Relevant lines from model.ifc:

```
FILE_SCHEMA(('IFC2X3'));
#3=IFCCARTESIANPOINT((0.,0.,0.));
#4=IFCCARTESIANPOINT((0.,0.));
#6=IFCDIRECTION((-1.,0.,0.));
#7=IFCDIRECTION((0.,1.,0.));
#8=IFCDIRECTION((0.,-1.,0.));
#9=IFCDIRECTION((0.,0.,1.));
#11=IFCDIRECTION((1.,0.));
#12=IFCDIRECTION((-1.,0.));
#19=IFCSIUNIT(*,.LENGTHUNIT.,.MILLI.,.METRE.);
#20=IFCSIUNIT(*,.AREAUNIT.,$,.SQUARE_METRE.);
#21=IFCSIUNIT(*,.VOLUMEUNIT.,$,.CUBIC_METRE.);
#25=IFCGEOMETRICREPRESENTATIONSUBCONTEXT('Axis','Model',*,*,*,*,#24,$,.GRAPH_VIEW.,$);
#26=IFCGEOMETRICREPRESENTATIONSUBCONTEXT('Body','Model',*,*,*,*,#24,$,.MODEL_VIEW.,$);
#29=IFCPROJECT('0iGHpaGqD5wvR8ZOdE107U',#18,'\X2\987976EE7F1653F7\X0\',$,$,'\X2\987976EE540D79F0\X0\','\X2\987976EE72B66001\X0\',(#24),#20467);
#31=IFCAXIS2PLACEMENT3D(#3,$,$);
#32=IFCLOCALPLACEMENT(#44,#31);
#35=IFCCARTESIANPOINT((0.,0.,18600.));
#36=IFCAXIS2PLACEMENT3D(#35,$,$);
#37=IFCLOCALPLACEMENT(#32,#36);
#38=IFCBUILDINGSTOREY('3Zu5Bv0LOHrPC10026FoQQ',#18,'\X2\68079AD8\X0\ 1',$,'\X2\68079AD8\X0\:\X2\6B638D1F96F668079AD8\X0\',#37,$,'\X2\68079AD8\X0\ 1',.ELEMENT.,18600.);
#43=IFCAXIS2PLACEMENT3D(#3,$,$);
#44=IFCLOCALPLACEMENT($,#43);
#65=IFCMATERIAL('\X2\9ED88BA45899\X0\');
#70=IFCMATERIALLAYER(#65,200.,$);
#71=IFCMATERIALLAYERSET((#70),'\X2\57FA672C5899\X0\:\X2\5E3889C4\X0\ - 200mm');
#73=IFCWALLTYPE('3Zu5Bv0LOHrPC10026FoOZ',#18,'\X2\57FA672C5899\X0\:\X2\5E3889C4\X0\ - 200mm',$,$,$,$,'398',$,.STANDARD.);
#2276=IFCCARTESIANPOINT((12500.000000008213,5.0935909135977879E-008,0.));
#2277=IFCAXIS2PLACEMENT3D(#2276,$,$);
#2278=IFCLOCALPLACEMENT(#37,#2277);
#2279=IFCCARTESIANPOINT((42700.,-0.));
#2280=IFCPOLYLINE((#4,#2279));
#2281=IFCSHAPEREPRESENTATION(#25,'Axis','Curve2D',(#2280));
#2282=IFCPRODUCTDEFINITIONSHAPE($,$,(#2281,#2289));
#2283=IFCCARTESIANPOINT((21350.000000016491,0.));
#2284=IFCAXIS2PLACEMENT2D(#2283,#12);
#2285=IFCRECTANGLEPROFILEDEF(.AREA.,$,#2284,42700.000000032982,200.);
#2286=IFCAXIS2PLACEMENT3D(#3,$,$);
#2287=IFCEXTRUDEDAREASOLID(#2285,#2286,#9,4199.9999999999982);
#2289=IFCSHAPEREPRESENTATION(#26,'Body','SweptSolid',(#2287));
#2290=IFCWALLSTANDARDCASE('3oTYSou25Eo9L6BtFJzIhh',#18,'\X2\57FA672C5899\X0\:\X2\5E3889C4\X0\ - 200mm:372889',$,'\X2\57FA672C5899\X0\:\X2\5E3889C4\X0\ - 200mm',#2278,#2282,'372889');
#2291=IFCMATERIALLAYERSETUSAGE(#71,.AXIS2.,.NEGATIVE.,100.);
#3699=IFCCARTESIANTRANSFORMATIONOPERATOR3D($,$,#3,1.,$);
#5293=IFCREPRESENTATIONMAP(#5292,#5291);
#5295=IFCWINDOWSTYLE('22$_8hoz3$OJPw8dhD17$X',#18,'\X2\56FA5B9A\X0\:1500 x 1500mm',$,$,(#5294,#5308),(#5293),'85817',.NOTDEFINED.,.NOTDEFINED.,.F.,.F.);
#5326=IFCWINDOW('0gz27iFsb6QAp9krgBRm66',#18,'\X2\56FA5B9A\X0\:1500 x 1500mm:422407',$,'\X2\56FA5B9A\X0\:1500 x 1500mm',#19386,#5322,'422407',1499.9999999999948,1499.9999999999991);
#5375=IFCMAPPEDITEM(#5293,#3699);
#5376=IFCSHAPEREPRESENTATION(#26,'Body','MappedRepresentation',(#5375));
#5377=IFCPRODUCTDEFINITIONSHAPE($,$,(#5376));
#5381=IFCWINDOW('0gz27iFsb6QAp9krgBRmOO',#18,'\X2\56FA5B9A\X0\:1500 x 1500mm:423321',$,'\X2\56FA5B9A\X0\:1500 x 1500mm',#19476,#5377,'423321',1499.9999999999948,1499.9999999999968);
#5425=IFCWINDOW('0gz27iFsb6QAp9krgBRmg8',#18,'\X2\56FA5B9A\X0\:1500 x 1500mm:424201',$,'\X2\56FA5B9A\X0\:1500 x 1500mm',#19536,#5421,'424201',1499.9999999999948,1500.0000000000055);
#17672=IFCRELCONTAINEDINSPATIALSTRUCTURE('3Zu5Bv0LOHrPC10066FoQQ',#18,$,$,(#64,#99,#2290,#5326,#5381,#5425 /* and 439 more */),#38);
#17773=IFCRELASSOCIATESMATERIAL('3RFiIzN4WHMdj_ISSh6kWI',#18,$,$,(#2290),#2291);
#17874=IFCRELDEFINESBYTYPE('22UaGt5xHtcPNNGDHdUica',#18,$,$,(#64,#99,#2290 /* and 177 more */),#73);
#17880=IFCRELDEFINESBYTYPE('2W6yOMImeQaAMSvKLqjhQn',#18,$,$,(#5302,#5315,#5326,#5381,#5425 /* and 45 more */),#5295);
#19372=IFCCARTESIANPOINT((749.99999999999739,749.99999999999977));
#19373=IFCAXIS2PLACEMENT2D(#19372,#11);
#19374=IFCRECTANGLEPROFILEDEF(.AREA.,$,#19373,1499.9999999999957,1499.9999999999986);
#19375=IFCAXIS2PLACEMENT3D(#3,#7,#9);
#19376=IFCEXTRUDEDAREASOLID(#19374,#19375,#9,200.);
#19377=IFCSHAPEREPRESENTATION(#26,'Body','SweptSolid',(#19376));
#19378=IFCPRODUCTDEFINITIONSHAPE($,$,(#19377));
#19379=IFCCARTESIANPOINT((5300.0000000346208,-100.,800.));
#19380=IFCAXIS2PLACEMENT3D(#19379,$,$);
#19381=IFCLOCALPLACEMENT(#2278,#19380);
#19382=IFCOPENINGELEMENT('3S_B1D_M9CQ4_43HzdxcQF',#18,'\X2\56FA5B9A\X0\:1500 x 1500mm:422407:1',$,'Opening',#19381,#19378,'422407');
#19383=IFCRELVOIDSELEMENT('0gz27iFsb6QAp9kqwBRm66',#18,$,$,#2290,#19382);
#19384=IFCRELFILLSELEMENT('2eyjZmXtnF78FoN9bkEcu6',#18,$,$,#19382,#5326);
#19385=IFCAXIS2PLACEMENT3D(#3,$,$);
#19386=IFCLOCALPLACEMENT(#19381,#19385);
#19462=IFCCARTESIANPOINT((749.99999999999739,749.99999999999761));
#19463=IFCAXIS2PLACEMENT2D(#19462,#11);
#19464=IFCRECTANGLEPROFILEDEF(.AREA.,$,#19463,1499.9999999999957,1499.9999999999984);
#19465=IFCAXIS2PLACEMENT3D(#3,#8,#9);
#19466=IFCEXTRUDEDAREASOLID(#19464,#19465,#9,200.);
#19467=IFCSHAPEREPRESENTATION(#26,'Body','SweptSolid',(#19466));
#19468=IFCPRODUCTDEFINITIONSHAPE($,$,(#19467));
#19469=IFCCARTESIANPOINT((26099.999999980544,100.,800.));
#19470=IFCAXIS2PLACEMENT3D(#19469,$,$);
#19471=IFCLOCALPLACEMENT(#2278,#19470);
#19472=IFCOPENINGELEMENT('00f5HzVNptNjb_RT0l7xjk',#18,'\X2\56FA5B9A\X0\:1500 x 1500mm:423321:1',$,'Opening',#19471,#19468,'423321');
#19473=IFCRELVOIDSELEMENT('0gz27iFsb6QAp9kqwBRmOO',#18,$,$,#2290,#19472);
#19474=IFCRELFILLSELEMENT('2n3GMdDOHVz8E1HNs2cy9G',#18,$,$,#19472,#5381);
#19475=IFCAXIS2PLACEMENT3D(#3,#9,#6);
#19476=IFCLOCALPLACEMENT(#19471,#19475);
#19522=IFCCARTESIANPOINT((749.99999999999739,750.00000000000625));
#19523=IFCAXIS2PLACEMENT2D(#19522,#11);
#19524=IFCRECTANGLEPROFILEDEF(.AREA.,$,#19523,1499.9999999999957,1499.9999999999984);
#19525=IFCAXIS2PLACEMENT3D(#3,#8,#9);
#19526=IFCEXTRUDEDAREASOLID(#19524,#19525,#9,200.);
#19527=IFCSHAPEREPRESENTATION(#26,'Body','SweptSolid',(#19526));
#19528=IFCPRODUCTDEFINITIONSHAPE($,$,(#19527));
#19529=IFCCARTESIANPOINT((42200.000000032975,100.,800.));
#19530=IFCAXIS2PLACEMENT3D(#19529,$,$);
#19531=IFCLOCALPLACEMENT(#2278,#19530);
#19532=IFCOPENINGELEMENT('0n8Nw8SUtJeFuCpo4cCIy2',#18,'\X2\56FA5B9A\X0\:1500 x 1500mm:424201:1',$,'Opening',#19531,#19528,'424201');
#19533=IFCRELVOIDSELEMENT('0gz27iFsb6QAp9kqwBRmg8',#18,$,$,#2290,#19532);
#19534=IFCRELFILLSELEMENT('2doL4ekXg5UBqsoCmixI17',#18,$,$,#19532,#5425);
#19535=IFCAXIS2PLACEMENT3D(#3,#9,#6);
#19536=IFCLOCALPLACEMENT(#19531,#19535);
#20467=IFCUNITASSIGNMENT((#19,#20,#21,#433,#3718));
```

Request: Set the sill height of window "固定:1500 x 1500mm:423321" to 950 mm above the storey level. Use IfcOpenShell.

```python
import numpy as np
import ifcopenshell
import ifcopenshell.api.geometry
import ifcopenshell.geom
import ifcopenshell.util.element
import ifcopenshell.util.placement
import ifcopenshell.util.shape
import ifcopenshell.util.unit

model = ifcopenshell.open("model.ifc")
unit_scale = ifcopenshell.util.unit.calculate_unit_scale(model)

window = model.by_guid("0gz27iFsb6QAp9krgBRmOO")
opening = window.FillsVoids[0].RelatingOpeningElement
storey = ifcopenshell.util.element.get_container(window, ifc_class="IfcBuildingStorey")
level = ifcopenshell.util.placement.get_local_placement(storey.ObjectPlacement)[2, 3]

# The opening's origin need not be at the sill, so measure its lowest point.
shape = ifcopenshell.geom.create_shape(ifcopenshell.geom.settings(), opening)
bottom = ifcopenshell.util.shape.get_shape_bottom_elevation(shape, shape.geometry) / unit_scale
dz = level + 0.95 / unit_scale - bottom

shift = np.array([0.0, 0.0, dz])
# The window is placed relative to its opening, so it follows when the opening moves.
matrix = ifcopenshell.util.placement.get_local_placement(opening.ObjectPlacement)
matrix[:3, 3] += shift
ifcopenshell.api.geometry.edit_object_placement(
    model, product=opening, matrix=matrix, is_si=False, should_transform_children=True
)

print(f"moved by {dz * unit_scale:+.3f} m")

model.write("model_updated.ifc")
```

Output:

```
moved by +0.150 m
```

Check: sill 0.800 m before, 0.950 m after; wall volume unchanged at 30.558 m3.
